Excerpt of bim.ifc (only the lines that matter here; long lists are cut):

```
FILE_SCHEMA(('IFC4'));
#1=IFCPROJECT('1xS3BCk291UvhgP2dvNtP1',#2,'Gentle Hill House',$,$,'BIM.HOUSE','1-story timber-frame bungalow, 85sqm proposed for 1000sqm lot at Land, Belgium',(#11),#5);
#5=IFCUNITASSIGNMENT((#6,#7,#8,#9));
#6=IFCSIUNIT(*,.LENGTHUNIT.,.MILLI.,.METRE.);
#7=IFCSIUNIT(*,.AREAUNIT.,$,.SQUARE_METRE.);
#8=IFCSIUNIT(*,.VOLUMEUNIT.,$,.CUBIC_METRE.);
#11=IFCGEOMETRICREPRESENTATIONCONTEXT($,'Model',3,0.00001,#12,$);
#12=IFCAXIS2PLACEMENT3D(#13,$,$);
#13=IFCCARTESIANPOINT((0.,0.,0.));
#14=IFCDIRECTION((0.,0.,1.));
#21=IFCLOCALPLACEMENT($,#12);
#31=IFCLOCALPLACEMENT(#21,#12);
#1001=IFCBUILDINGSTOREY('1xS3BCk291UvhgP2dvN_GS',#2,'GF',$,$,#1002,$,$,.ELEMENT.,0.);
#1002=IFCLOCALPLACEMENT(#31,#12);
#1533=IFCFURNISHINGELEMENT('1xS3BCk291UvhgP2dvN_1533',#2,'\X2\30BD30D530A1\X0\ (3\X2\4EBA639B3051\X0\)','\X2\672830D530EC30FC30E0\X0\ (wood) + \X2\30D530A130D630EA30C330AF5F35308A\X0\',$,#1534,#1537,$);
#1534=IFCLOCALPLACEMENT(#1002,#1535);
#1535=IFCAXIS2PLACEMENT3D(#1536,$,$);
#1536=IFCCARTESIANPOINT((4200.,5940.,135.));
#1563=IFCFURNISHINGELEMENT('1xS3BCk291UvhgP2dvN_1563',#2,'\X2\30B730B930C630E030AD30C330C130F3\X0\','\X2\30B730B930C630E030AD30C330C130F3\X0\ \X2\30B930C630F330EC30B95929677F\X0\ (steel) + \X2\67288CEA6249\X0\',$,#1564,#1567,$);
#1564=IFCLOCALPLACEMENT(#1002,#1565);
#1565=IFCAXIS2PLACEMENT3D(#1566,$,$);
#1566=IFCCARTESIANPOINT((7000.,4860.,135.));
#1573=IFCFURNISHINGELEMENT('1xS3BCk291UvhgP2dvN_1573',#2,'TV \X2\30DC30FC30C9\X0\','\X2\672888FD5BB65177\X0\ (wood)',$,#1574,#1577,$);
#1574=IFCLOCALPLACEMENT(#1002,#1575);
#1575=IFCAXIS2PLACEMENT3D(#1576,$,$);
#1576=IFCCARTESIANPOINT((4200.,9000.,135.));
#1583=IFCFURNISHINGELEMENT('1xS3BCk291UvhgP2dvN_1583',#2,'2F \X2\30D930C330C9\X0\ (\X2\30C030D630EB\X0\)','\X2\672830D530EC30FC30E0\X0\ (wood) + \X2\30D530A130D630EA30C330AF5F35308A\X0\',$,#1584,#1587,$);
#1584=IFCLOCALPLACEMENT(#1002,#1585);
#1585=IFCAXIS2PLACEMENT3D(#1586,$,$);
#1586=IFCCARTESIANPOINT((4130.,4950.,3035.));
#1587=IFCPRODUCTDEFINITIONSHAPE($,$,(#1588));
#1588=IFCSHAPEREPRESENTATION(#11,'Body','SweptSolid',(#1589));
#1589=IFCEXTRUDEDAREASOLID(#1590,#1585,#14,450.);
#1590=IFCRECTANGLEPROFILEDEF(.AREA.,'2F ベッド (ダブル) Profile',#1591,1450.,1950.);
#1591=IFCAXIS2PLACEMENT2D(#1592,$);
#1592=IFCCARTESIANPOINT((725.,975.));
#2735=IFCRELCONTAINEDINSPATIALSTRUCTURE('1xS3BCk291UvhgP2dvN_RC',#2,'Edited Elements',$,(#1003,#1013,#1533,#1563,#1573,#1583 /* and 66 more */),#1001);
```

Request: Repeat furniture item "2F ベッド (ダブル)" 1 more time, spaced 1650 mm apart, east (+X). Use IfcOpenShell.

```python
import numpy as np
import ifcopenshell
import ifcopenshell.api.geometry
import ifcopenshell.api.root
import ifcopenshell.util.element
import ifcopenshell.util.placement

model = ifcopenshell.open("bim.ifc")


def reuse_history(source, copy):
    """copy_class also copies each property set's owner history, people and application; keep the originals."""
    for rel in copy.IsDefinedBy:
        if rel.is_a("IfcRelDefinesByProperties") and (history := rel.RelatingPropertyDefinition.OwnerHistory):
            rel.RelatingPropertyDefinition.OwnerHistory = source.OwnerHistory
            ifcopenshell.util.element.remove_deep2(model, history)


source = model.by_id(1583)
base = ifcopenshell.util.placement.get_local_placement(source.ObjectPlacement)
step = np.array([1.0, 0.0, 0.0]) * 1650.0

for i in range(1, 2):
    copy = ifcopenshell.api.root.copy_class(model, product=source)
    copy.Representation = ifcopenshell.util.element.copy_deep(
        model, source.Representation, exclude=["IfcGeometricRepresentationContext", "IfcRepresentationMap"]
    )
    reuse_history(source, copy)
    matrix = base.copy()
    matrix[:3, 3] += i * step
    print("added at", matrix[:3, 3].round(3) + 0.0)
    ifcopenshell.api.geometry.edit_object_placement(model, product=copy, matrix=matrix, is_si=False)

model.write("bim_v2.ifc")
```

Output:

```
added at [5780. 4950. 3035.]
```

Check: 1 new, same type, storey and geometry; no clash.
